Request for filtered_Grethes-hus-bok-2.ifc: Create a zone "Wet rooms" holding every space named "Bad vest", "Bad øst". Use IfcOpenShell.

First a look at what the model holds.

```python
import ifcopenshell

model = ifcopenshell.open("filtered_Grethes-hus-bok-2.ifc")
print(model.schema)
seen = {}
for space in model.by_type("IfcSpace"):
    seen[space.LongName] = seen.get(space.LongName, 0) + 1
for name, count in sorted(seen.items(), key=str):
    print(count, "x", name)
print("zones:", [z.Name for z in model.by_type("IfcZone")][:20])
```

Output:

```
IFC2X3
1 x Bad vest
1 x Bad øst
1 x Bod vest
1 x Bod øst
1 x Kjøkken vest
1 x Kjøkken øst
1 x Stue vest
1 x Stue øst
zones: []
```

```python
import ifcopenshell
import ifcopenshell.api.group
import ifcopenshell.api.root

model = ifcopenshell.open("filtered_Grethes-hus-bok-2.ifc")

names = {"Bad vest", "Bad øst"}
spaces = [s for s in model.by_type("IfcSpace") if s.LongName in names]

zone = ifcopenshell.api.root.create_entity(model, ifc_class="IfcZone", name="Wet rooms")
ifcopenshell.api.group.assign_group(model, products=spaces, group=zone)
print(len(spaces), "spaces in", zone.Name)

model.write("filtered_Grethes-hus-bok-2_v2.ifc")
```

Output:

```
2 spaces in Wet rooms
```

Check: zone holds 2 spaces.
